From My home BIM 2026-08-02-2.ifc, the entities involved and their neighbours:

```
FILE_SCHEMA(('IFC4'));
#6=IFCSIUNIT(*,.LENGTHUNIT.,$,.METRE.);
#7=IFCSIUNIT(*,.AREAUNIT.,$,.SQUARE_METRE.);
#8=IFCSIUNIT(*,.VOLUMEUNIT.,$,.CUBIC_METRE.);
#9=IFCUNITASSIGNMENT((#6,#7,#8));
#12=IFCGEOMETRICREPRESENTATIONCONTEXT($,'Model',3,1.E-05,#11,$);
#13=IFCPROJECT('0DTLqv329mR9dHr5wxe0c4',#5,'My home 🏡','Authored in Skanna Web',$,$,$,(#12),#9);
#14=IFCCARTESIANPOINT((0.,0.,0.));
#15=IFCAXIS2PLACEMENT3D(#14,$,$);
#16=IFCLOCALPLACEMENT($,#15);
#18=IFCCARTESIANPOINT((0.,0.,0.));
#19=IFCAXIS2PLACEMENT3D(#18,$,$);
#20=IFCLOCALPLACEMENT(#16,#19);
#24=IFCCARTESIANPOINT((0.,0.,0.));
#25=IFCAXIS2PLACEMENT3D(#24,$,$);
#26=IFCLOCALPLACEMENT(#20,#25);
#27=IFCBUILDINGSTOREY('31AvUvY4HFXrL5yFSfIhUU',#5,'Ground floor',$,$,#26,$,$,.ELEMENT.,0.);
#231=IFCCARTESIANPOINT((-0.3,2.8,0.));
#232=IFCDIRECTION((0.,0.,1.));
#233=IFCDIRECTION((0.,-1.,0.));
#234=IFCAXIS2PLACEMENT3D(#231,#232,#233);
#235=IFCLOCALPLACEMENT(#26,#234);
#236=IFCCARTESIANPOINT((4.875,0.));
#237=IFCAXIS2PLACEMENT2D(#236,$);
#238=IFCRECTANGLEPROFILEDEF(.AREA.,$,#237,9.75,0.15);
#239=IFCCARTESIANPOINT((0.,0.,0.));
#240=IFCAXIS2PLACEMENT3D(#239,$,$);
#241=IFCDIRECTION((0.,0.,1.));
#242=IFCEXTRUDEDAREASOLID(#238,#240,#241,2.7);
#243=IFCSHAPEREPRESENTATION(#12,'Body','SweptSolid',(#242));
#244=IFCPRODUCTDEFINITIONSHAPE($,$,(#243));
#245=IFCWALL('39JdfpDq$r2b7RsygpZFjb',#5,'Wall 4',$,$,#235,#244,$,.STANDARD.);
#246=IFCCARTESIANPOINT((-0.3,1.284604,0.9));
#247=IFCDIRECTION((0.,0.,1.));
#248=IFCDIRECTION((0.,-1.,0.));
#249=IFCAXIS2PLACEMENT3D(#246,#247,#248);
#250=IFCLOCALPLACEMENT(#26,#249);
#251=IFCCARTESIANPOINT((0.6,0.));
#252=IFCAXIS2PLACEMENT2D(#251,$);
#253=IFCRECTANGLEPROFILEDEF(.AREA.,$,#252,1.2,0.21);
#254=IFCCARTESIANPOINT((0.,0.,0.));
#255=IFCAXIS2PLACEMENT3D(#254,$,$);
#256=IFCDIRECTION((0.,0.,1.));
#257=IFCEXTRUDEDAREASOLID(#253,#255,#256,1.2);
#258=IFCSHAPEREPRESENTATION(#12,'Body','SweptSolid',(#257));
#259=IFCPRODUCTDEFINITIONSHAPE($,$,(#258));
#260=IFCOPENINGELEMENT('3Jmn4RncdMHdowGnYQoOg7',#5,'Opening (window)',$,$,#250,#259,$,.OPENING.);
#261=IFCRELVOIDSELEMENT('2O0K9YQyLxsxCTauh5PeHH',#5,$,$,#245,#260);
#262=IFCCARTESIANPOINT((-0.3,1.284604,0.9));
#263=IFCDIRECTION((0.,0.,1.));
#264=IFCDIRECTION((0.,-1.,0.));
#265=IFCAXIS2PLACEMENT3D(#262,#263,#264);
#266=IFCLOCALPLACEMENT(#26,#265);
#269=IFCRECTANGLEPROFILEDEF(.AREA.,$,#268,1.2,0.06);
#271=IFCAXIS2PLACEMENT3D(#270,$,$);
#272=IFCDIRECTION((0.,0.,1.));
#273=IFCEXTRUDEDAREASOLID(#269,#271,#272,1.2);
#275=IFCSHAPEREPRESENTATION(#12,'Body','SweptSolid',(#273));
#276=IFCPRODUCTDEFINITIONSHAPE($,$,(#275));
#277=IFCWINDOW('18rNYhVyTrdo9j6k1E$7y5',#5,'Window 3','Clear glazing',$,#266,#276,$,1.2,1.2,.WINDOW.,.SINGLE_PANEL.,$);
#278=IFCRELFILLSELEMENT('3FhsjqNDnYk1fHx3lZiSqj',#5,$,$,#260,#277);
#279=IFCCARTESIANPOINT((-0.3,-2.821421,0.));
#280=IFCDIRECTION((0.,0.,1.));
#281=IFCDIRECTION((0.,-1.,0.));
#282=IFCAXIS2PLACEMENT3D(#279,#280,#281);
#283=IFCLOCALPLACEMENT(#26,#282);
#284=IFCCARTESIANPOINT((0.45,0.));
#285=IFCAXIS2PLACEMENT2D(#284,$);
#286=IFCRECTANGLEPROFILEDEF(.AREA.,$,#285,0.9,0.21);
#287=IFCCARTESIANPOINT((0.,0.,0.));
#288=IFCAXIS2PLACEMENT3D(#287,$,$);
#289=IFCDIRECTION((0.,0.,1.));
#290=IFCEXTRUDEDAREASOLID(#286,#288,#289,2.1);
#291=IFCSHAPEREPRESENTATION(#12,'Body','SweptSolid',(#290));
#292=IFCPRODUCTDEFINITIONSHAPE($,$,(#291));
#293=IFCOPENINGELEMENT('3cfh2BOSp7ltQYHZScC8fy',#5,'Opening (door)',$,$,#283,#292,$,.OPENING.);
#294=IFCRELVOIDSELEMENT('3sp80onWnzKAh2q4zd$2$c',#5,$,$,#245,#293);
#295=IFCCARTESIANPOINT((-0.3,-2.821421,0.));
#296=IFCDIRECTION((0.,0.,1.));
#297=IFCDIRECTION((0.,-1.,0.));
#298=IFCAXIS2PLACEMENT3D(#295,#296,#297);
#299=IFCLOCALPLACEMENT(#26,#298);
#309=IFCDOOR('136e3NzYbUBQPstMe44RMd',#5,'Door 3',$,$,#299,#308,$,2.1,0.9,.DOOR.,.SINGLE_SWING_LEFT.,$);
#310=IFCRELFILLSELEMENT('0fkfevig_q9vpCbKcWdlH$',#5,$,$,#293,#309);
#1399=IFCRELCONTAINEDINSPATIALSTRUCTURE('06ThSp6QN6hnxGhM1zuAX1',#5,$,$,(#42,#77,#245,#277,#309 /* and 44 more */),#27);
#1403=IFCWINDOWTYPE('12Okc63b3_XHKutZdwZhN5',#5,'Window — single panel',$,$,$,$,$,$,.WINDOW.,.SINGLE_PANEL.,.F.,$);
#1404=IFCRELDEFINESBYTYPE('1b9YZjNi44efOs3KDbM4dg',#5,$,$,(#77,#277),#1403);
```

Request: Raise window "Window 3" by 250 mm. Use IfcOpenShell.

```python
import numpy as np
import ifcopenshell
import ifcopenshell.api.geometry
import ifcopenshell.util.placement
import ifcopenshell.util.unit

model = ifcopenshell.open("My home BIM 2026-08-02-2.ifc")
unit_scale = ifcopenshell.util.unit.calculate_unit_scale(model)

window = model.by_guid("18rNYhVyTrdo9j6k1E$7y5")
opening = window.FillsVoids[0].RelatingOpeningElement
dz = 0.25

shift = np.array([0.0, 0.0, dz])
# The window is not placed relative to its opening, so move both.
for product in (opening, window):
    matrix = ifcopenshell.util.placement.get_local_placement(product.ObjectPlacement)
    matrix[:3, 3] += shift
    ifcopenshell.api.geometry.edit_object_placement(model, product=product, matrix=matrix, is_si=False)

print(f"moved by {dz * unit_scale:+.3f} m")

model.write("My home BIM 2026-08-02-2_updated.ifc")
```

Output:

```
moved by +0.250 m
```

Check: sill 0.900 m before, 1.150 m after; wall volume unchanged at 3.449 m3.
